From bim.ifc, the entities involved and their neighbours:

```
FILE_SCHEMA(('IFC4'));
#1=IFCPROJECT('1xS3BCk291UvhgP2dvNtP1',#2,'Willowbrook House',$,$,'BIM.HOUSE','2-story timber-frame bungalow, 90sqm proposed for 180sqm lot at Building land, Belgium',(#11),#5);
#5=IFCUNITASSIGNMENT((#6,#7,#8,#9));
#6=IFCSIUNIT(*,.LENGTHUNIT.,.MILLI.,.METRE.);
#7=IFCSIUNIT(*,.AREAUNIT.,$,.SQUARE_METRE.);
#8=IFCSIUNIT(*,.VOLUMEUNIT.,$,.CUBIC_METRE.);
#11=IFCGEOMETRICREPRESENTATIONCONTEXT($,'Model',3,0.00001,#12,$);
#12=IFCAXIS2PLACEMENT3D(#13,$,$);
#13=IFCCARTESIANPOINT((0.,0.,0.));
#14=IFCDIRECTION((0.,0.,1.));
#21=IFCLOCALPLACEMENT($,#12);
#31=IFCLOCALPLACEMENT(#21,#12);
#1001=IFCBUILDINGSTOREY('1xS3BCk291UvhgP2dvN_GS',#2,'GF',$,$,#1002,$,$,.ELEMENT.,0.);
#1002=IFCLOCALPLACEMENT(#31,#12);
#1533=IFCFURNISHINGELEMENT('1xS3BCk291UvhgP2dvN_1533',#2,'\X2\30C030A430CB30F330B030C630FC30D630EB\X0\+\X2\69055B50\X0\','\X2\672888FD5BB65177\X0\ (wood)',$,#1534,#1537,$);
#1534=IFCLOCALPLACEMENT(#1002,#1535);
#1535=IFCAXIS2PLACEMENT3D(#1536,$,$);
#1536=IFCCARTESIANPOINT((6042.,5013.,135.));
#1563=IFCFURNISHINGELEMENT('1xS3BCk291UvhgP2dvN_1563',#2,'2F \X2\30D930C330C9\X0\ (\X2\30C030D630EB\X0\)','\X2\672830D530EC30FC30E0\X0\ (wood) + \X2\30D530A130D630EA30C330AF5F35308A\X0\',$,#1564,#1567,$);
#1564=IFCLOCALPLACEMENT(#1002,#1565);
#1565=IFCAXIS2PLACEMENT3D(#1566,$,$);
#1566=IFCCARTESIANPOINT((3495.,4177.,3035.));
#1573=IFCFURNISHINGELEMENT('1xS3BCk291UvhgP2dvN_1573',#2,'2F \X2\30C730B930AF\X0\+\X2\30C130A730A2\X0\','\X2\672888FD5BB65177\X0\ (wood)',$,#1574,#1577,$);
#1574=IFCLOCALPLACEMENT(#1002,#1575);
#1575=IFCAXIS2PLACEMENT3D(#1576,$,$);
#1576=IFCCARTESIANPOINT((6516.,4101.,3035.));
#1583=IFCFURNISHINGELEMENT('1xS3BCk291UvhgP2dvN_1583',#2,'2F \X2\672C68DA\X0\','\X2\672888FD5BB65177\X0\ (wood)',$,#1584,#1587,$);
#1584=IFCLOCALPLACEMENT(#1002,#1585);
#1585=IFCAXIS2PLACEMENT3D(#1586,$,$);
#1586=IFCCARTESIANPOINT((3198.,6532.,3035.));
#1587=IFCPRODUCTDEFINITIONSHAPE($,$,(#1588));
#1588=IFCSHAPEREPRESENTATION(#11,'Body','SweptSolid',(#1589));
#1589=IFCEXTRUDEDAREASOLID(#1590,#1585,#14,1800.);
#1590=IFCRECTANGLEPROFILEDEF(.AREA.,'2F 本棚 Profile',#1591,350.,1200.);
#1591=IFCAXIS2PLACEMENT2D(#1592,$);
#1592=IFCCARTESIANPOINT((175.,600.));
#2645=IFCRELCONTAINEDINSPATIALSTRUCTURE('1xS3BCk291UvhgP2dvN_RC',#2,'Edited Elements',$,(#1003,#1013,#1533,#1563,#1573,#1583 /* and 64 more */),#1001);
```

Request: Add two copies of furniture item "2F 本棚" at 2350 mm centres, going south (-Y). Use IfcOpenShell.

```python
import numpy as np
import ifcopenshell
import ifcopenshell.api.geometry
import ifcopenshell.api.root
import ifcopenshell.util.element
import ifcopenshell.util.placement
import ifcopenshell.util.unit

model = ifcopenshell.open("bim.ifc")
unit_scale = ifcopenshell.util.unit.calculate_unit_scale(model)


def reuse_history(source, copy):
    """copy_class also copies each property set's owner history, people and application; keep the originals."""
    for rel in copy.IsDefinedBy:
        if rel.is_a("IfcRelDefinesByProperties") and (history := rel.RelatingPropertyDefinition.OwnerHistory):
            rel.RelatingPropertyDefinition.OwnerHistory = source.OwnerHistory
            ifcopenshell.util.element.remove_deep2(model, history)


source = model.by_guid("1xS3BCk291UvhgP2dvN_1583")
base = ifcopenshell.util.placement.get_local_placement(source.ObjectPlacement)
step = np.array([0.0, -1.0, 0.0]) * 2.35 / unit_scale

for i in range(1, 3):
    copy = ifcopenshell.api.root.copy_class(model, product=source)
    copy.Representation = ifcopenshell.util.element.copy_deep(
        model, source.Representation, exclude=["IfcGeometricRepresentationContext", "IfcRepresentationMap"]
    )
    reuse_history(source, copy)
    matrix = base.copy()
    matrix[:3, 3] += i * step
    print("added at", matrix[:3, 3].round(3) + 0.0)
    ifcopenshell.api.geometry.edit_object_placement(model, product=copy, matrix=matrix, is_si=False)

model.write("bim_edited.ifc")
```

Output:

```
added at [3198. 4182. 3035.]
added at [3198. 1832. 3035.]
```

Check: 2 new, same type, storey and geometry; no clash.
